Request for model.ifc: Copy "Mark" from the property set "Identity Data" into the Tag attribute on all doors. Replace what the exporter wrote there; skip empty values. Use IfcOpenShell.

First a look at what the model holds.

```python
import ifcopenshell
import ifcopenshell.util.element

model = ifcopenshell.open("model.ifc")
print(model.schema)
doors = model.by_type("IfcDoor")
print(len(doors), "doors")
for e in doors[:8]:
    source = ifcopenshell.util.element.get_pset(e, "Identity Data", "Mark")
    target = e.Tag
    print(e.id(), repr(source), repr(target), sep=" | ")
```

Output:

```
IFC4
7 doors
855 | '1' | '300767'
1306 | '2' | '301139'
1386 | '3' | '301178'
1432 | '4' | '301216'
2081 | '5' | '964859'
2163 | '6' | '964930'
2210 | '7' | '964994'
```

```python
import ifcopenshell
import ifcopenshell.util.element

model = ifcopenshell.open("model.ifc")

count = 0
for e in model.by_type("IfcDoor"):
    value = ifcopenshell.util.element.get_pset(e, "Identity Data", "Mark")
    current = e.Tag
    if not value or not value.strip() or current == value:
        continue
    e.Tag = value
    count += 1

print(count, "doors updated")

model.write("model_updated.ifc")
```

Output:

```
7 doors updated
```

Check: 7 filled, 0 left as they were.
